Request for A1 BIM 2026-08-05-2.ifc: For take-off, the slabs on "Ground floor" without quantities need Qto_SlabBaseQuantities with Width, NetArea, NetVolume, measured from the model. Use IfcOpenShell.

First a look at what the model holds.

```python
import ifcopenshell
import ifcopenshell.util.element
import ifcopenshell.util.unit

model = ifcopenshell.open("A1 BIM 2026-08-05-2.ifc")
print(model.schema)
for unit_type in ("LENGTHUNIT", "AREAUNIT", "VOLUMEUNIT"):
    print(unit_type, ifcopenshell.util.unit.calculate_unit_scale(model, unit_type))
storey = next(s for s in model.by_type("IfcBuildingStorey") if s.Name == "Ground floor")
slabs = [e for e in ifcopenshell.util.element.get_decomposition(storey) if e.is_a("IfcSlab")]
for e in sorted(slabs, key=lambda e: e.id()):
    print(e.id(), e.is_a(), e.Name, list(ifcopenshell.util.element.get_psets(e, qtos_only=True)), sep=" | ")
```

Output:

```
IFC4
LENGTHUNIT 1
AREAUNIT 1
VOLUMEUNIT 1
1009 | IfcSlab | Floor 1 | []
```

```python
import ifcopenshell
import ifcopenshell.api.pset
import ifcopenshell.geom
import ifcopenshell.util.element
import ifcopenshell.util.shape
import ifcopenshell.util.unit

model = ifcopenshell.open("A1 BIM 2026-08-05-2.ifc")
unit_scale = ifcopenshell.util.unit.calculate_unit_scale(model)
area_scale = ifcopenshell.util.unit.calculate_unit_scale(model, "AREAUNIT")
volume_scale = ifcopenshell.util.unit.calculate_unit_scale(model, "VOLUMEUNIT")
settings = ifcopenshell.geom.settings()

storey = next(s for s in model.by_type("IfcBuildingStorey") if s.Name == "Ground floor")
slabs = [e for e in ifcopenshell.util.element.get_decomposition(storey) if e.is_a("IfcSlab")]

for e in sorted(slabs, key=lambda e: e.id()):
    if ifcopenshell.util.element.get_psets(e, qtos_only=True, should_inherit=False):
        continue
    # Geometry comes back in metres, in the element's own axes.
    shape = ifcopenshell.geom.create_shape(settings, e)
    values = {
        "Width": ifcopenshell.util.shape.get_z(shape.geometry) / unit_scale,
        "NetArea": ifcopenshell.util.shape.get_footprint_area(shape.geometry) / area_scale,
        "NetVolume": ifcopenshell.util.shape.get_volume(shape.geometry) / volume_scale,
    }
    qto = ifcopenshell.api.pset.add_qto(model, product=e, name="Qto_SlabBaseQuantities")
    ifcopenshell.api.pset.edit_qto(model, qto=qto, properties=values)
    print(e.id(), {k: round(v, 3) for k, v in values.items()})

model.write("A1 BIM 2026-08-05-2_edited.ifc")
```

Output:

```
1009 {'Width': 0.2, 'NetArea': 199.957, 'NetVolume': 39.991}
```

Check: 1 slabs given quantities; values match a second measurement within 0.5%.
